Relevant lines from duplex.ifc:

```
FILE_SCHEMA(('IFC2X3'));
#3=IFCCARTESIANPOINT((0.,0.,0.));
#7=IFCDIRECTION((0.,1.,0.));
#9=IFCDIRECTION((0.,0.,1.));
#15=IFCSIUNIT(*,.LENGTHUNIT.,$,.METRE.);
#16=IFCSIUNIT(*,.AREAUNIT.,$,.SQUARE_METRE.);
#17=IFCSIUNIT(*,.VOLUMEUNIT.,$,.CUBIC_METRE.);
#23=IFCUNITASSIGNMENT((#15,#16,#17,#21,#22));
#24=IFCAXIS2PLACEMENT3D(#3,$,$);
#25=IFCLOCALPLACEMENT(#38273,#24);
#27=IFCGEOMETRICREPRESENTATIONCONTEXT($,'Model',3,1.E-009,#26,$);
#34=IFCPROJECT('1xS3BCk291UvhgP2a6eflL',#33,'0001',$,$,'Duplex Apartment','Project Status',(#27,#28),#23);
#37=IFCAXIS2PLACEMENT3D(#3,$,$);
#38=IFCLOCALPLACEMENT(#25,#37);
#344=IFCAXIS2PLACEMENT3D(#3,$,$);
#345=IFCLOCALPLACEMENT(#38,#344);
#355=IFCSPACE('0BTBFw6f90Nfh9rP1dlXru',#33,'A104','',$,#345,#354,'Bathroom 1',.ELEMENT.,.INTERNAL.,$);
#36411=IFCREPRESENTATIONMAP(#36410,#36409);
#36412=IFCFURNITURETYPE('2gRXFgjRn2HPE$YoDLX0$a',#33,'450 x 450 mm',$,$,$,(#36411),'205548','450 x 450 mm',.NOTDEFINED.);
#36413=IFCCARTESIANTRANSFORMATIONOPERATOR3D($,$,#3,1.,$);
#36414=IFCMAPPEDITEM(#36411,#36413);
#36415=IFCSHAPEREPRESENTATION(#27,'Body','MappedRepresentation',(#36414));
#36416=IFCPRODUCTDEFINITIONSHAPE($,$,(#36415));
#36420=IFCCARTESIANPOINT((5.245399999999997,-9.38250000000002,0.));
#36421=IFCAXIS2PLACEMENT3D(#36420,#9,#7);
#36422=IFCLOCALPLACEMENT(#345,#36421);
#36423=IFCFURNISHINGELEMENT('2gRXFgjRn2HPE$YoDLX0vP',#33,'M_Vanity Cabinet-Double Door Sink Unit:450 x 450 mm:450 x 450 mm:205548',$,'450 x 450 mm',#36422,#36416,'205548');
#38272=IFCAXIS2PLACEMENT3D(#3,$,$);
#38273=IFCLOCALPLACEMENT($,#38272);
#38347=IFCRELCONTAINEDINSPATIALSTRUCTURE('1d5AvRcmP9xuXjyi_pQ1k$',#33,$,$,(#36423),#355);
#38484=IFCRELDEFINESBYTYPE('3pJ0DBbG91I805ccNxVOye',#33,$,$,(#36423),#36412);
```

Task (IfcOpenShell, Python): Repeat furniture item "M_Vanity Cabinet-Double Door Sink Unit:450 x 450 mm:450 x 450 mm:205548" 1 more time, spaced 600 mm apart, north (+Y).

```python
import numpy as np
import ifcopenshell
import ifcopenshell.api.geometry
import ifcopenshell.api.root
import ifcopenshell.util.element
import ifcopenshell.util.placement

model = ifcopenshell.open("duplex.ifc")


def reuse_history(source, copy):
    """copy_class also copies each property set's owner history, people and application; keep the originals."""
    for rel in copy.IsDefinedBy:
        if rel.is_a("IfcRelDefinesByProperties") and (history := rel.RelatingPropertyDefinition.OwnerHistory):
            rel.RelatingPropertyDefinition.OwnerHistory = source.OwnerHistory
            ifcopenshell.util.element.remove_deep2(model, history)


source = model.by_guid("2gRXFgjRn2HPE$YoDLX0vP")
base = ifcopenshell.util.placement.get_local_placement(source.ObjectPlacement)
step = np.array([0.0, 1.0, 0.0]) * 0.6

for i in range(1, 2):
    copy = ifcopenshell.api.root.copy_class(model, product=source)
    copy.Representation = ifcopenshell.util.element.copy_deep(
        model, source.Representation, exclude=["IfcGeometricRepresentationContext", "IfcRepresentationMap"]
    )
    copy.Name = "M_Vanity Cabinet-Double Door Sink Unit:450 x 450 mm:450 x 450 mm"
    copy.Tag = None
    reuse_history(source, copy)
    matrix = base.copy()
    matrix[:3, 3] += i * step
    print("added at", matrix[:3, 3].round(3) + 0.0)
    ifcopenshell.api.geometry.edit_object_placement(model, product=copy, matrix=matrix, is_si=False)

model.write("duplex_v2.ifc")
```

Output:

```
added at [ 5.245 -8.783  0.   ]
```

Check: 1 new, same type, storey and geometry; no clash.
